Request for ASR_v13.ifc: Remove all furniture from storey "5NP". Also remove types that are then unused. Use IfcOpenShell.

First a look at what the model holds.

```python
import ifcopenshell
import ifcopenshell.util.element

model = ifcopenshell.open("ASR_v13.ifc")
print(model.schema)
storey = next(s for s in model.by_type("IfcBuildingStorey") if s.Name == "5NP")
furniture = [e for e in ifcopenshell.util.element.get_decomposition(storey) if e.is_a("IfcFurnishingElement")]
seen = {}
for e in furniture:
    element_type = ifcopenshell.util.element.get_type(e)
    name = element_type.Name if element_type not in (None, e) else None
    seen[name] = seen.get(name, 0) + 1
for name, count in sorted(seen.items(), key=str):
    print(count, "x", name)
```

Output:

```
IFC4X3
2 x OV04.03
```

```python
import ifcopenshell
import ifcopenshell.api.root
import ifcopenshell.util.element

model = ifcopenshell.open("ASR_v13.ifc")

storey = next(s for s in model.by_type("IfcBuildingStorey") if s.Name == "5NP")
furniture = [e for e in ifcopenshell.util.element.get_decomposition(storey) if e.is_a("IfcFurnishingElement")]
types = {ifcopenshell.util.element.get_type(e) for e in furniture} - {None, *furniture}

for e in furniture:
    ifcopenshell.api.root.remove_product(model, product=e)
print(len(furniture), "removed")

unused = [t for t in types if not ifcopenshell.util.element.get_types(t)]
for t in unused:
    ifcopenshell.api.root.remove_product(model, product=t)
print(len(unused), "unused types removed")

model.write("ASR_v13_edited.ifc")
```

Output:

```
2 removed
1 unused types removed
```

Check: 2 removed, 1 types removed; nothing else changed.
